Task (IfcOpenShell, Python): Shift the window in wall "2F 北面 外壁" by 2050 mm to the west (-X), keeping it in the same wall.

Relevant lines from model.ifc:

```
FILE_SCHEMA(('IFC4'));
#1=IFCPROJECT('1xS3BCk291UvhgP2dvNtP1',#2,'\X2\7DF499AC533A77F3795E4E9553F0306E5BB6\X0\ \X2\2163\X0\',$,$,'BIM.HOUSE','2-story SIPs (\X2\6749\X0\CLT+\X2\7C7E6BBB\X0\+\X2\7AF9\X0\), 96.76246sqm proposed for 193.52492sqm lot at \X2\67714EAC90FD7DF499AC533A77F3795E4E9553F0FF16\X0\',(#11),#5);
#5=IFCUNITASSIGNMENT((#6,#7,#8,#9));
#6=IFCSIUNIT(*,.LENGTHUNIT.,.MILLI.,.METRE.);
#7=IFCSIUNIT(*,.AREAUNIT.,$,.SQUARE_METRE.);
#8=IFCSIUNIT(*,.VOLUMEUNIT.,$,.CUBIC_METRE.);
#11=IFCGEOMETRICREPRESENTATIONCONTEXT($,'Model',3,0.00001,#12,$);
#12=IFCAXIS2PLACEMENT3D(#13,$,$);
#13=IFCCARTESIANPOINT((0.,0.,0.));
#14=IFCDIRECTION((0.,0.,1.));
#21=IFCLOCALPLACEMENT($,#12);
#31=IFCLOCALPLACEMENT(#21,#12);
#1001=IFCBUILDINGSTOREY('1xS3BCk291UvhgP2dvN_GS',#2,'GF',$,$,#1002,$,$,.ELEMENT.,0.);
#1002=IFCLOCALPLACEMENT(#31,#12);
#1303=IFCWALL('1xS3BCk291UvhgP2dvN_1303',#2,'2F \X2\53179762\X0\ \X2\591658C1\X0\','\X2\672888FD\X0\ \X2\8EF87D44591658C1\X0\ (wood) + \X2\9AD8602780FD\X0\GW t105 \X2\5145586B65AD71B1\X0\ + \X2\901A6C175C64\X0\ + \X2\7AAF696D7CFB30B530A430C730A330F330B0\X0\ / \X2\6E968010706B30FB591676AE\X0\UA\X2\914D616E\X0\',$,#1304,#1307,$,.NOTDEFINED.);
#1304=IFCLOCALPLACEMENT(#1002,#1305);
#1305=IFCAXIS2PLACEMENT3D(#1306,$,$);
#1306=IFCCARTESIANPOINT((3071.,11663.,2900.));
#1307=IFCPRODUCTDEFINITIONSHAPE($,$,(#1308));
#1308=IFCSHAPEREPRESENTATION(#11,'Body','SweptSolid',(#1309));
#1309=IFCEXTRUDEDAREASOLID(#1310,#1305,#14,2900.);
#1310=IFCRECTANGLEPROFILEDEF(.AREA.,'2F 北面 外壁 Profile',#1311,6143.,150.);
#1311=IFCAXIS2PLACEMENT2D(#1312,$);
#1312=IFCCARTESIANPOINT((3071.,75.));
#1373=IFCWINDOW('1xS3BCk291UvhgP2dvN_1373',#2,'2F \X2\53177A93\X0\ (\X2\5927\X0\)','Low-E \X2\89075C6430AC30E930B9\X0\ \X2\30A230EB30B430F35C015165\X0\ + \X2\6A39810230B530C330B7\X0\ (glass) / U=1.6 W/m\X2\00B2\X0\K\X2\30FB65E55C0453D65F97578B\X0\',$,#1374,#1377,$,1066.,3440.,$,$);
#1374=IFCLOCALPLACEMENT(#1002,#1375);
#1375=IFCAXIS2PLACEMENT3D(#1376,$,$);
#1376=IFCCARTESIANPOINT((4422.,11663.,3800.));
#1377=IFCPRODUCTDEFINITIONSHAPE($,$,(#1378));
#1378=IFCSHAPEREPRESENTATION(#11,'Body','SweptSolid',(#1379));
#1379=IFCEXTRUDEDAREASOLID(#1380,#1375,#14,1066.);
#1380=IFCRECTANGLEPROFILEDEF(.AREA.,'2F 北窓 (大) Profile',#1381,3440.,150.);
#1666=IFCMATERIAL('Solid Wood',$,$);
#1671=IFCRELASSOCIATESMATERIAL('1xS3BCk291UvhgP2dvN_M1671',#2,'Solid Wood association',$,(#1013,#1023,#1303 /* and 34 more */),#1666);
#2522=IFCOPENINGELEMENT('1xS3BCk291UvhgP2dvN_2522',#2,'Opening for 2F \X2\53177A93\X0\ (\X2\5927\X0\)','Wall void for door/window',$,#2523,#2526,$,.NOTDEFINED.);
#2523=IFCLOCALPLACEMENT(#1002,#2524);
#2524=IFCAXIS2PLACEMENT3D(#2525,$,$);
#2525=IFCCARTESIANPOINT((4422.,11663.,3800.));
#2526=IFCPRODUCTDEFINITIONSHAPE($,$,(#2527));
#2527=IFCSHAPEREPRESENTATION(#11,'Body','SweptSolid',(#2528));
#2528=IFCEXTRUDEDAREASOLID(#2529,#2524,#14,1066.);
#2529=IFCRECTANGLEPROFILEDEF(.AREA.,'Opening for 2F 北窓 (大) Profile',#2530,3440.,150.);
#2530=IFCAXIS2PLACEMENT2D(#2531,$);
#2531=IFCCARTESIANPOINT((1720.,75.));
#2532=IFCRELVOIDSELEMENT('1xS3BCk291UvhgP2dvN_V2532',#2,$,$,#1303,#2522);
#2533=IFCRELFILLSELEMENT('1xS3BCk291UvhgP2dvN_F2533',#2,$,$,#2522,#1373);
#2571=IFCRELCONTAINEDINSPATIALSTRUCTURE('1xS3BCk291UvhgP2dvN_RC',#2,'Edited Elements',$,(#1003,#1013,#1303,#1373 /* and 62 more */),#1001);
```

```python
import ifcopenshell
import ifcopenshell.api.geometry
import ifcopenshell.util.placement
import ifcopenshell.util.unit

model = ifcopenshell.open("model.ifc")
unit_scale = ifcopenshell.util.unit.calculate_unit_scale(model)

window = model.by_id(1373)
opening = window.FillsVoids[0].RelatingOpeningElement
wall = opening.VoidsElements[0].RelatingBuildingElement

wall_matrix = ifcopenshell.util.placement.get_local_placement(wall.ObjectPlacement)
shift = wall_matrix[:3, 0] * -2.05 / unit_scale
before = ifcopenshell.util.placement.get_local_placement(window.ObjectPlacement)[:3, 3].copy()

# The window is not placed relative to its opening, so move both.
for product in (opening, window):
    matrix = ifcopenshell.util.placement.get_local_placement(product.ObjectPlacement)
    matrix[:3, 3] += shift
    ifcopenshell.api.geometry.edit_object_placement(model, product=product, matrix=matrix, is_si=False)

after = ifcopenshell.util.placement.get_local_placement(window.ObjectPlacement)[:3, 3]
print("window moved by", (after - before).round(3) + 0.0)

model.write("model-out.ifc")
```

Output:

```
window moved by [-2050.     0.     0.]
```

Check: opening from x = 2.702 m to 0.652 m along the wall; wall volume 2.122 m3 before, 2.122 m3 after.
